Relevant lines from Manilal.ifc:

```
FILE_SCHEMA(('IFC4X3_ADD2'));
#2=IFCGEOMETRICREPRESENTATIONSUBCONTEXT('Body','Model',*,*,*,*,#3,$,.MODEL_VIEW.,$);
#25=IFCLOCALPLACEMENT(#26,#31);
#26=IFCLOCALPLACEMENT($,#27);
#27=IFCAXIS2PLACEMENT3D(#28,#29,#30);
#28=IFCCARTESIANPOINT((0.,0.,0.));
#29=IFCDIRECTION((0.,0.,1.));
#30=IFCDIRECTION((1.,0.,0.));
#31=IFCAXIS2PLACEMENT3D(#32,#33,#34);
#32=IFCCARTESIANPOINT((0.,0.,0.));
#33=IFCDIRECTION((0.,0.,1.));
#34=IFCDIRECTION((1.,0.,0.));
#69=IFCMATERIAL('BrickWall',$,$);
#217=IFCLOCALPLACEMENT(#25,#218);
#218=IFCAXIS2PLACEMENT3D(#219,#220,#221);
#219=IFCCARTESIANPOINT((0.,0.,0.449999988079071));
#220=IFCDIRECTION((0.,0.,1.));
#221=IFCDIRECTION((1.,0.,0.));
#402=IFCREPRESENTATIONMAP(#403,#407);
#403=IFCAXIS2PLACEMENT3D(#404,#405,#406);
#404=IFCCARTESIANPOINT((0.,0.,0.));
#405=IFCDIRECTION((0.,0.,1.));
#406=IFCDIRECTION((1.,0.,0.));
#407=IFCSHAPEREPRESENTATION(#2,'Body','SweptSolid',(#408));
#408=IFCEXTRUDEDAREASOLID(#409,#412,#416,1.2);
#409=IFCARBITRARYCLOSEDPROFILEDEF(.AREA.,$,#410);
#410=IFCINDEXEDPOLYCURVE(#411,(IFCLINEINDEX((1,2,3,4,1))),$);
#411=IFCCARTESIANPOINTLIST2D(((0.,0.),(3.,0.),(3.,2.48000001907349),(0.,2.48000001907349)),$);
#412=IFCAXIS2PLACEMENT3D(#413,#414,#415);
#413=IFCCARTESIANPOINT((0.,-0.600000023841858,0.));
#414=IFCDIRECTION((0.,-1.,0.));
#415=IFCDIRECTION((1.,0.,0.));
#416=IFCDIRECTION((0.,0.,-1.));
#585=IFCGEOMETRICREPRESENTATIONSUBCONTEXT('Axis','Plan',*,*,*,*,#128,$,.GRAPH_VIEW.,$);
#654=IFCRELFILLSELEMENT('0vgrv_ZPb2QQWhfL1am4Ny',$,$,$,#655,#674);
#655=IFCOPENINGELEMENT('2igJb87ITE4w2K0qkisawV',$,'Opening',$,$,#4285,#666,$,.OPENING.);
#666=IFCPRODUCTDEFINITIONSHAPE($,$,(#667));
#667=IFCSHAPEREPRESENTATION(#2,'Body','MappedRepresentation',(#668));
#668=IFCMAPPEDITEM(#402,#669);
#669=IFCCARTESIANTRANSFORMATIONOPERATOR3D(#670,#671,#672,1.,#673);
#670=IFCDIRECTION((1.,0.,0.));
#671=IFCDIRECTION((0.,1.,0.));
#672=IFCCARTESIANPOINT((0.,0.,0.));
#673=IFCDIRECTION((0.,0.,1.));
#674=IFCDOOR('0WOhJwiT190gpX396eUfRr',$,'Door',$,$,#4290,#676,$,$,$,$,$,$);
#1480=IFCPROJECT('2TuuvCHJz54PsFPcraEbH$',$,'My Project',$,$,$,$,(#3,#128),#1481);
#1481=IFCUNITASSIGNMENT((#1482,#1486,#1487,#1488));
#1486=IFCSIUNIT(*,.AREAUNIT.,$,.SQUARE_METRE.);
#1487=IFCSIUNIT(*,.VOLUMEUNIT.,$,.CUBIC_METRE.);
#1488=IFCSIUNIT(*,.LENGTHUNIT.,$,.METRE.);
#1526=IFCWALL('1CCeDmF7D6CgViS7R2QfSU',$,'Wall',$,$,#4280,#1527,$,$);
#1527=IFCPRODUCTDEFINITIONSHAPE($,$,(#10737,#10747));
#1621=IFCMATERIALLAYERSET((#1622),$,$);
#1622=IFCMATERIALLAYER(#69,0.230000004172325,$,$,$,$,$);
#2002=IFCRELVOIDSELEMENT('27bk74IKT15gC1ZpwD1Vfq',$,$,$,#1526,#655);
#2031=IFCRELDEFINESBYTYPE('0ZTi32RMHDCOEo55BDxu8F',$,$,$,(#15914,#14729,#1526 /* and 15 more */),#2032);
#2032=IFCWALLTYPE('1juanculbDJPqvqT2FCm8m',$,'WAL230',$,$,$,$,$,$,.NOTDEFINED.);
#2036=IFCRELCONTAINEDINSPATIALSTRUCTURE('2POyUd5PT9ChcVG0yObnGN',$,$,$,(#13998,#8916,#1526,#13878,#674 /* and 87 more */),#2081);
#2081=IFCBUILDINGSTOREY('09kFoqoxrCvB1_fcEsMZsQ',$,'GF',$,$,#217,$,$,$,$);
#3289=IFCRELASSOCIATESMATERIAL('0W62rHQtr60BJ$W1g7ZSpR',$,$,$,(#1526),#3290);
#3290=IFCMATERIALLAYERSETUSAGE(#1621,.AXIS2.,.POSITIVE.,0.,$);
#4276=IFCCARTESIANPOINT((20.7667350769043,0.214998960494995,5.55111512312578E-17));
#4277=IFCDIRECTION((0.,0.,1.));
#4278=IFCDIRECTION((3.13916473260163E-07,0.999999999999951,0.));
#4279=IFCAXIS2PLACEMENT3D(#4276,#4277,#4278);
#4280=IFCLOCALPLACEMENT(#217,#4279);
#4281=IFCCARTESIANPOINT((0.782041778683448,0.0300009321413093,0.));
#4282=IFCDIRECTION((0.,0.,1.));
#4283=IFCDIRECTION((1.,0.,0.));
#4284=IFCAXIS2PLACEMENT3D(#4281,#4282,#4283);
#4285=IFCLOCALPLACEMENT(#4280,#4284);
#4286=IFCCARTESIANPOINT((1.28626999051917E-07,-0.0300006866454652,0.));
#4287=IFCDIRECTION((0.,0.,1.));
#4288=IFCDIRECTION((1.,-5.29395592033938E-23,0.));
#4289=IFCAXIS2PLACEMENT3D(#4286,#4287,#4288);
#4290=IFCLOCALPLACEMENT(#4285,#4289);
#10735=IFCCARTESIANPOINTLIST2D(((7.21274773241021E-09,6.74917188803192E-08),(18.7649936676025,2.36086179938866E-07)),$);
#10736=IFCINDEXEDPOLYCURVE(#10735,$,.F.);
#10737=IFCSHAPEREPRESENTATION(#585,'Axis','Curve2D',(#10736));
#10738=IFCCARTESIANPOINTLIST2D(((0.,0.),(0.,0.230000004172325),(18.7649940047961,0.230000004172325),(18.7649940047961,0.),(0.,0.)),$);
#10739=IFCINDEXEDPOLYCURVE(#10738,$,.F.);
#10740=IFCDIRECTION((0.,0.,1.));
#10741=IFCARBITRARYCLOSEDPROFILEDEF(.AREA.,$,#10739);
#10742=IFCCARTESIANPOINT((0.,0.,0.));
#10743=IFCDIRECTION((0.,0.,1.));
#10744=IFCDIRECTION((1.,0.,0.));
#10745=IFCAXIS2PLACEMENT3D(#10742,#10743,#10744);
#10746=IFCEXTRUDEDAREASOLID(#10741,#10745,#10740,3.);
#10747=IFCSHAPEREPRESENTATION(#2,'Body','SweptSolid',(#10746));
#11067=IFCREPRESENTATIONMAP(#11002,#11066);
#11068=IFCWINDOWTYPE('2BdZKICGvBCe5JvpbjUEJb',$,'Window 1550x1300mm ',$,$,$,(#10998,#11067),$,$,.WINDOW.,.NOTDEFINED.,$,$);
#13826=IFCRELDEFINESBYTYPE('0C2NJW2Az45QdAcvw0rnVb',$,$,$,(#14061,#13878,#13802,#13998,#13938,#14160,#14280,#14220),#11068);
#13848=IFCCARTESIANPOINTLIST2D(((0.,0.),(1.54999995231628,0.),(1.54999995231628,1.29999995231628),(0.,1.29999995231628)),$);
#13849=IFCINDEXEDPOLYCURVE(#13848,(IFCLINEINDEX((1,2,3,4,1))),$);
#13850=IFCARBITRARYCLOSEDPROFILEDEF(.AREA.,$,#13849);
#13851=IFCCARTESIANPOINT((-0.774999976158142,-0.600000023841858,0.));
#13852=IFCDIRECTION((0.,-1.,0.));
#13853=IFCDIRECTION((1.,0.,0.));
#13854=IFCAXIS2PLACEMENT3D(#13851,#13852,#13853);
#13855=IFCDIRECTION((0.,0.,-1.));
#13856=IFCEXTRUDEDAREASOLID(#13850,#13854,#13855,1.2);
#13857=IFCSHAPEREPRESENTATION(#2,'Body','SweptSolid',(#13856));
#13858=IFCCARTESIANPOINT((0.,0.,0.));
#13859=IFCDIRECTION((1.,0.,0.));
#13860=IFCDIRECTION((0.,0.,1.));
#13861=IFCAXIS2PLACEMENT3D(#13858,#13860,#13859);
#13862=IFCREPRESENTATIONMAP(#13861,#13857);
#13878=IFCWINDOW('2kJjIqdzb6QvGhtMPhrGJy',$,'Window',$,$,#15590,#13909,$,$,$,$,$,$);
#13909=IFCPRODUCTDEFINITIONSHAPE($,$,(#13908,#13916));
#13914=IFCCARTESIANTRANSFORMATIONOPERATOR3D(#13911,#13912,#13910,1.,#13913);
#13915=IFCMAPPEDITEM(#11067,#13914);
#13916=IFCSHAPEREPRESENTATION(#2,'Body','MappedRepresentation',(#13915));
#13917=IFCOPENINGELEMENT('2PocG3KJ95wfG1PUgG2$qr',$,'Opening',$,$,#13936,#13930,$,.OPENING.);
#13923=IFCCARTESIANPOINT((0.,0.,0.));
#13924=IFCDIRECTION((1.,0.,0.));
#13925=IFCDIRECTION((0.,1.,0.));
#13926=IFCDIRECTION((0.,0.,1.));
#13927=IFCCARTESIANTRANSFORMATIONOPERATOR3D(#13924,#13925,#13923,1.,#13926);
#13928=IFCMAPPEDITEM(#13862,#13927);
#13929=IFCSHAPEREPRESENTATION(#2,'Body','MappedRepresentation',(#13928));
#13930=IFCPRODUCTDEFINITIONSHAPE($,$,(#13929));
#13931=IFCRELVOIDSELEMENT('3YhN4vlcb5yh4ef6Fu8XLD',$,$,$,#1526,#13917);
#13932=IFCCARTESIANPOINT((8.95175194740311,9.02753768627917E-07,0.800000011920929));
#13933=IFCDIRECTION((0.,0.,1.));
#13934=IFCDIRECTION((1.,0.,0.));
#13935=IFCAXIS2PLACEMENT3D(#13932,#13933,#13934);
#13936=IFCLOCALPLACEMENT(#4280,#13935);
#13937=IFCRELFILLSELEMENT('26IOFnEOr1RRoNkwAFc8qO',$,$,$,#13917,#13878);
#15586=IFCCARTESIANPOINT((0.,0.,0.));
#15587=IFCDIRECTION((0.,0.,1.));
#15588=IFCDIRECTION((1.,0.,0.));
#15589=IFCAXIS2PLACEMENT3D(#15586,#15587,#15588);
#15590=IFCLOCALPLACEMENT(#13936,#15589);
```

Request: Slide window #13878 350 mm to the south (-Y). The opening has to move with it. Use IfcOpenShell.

```python
import ifcopenshell
import ifcopenshell.api.geometry
import ifcopenshell.util.placement
import ifcopenshell.util.unit

model = ifcopenshell.open("Manilal.ifc")
unit_scale = ifcopenshell.util.unit.calculate_unit_scale(model)

window = model.by_id(13878)
opening = window.FillsVoids[0].RelatingOpeningElement
wall = opening.VoidsElements[0].RelatingBuildingElement

wall_matrix = ifcopenshell.util.placement.get_local_placement(wall.ObjectPlacement)
shift = wall_matrix[:3, 0] * -0.35 / unit_scale
before = ifcopenshell.util.placement.get_local_placement(window.ObjectPlacement)[:3, 3].copy()

# The window is placed relative to its opening, so it follows when the opening moves.
matrix = ifcopenshell.util.placement.get_local_placement(opening.ObjectPlacement)
matrix[:3, 3] += shift
ifcopenshell.api.geometry.edit_object_placement(
    model, product=opening, matrix=matrix, is_si=False, should_transform_children=True
)

after = ifcopenshell.util.placement.get_local_placement(window.ObjectPlacement)[:3, 3]
print("window moved by", (after - before).round(3) + 0.0)

model.write("Manilal_edited.ifc")
```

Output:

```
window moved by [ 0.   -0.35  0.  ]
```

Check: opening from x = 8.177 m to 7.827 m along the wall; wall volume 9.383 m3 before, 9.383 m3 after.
